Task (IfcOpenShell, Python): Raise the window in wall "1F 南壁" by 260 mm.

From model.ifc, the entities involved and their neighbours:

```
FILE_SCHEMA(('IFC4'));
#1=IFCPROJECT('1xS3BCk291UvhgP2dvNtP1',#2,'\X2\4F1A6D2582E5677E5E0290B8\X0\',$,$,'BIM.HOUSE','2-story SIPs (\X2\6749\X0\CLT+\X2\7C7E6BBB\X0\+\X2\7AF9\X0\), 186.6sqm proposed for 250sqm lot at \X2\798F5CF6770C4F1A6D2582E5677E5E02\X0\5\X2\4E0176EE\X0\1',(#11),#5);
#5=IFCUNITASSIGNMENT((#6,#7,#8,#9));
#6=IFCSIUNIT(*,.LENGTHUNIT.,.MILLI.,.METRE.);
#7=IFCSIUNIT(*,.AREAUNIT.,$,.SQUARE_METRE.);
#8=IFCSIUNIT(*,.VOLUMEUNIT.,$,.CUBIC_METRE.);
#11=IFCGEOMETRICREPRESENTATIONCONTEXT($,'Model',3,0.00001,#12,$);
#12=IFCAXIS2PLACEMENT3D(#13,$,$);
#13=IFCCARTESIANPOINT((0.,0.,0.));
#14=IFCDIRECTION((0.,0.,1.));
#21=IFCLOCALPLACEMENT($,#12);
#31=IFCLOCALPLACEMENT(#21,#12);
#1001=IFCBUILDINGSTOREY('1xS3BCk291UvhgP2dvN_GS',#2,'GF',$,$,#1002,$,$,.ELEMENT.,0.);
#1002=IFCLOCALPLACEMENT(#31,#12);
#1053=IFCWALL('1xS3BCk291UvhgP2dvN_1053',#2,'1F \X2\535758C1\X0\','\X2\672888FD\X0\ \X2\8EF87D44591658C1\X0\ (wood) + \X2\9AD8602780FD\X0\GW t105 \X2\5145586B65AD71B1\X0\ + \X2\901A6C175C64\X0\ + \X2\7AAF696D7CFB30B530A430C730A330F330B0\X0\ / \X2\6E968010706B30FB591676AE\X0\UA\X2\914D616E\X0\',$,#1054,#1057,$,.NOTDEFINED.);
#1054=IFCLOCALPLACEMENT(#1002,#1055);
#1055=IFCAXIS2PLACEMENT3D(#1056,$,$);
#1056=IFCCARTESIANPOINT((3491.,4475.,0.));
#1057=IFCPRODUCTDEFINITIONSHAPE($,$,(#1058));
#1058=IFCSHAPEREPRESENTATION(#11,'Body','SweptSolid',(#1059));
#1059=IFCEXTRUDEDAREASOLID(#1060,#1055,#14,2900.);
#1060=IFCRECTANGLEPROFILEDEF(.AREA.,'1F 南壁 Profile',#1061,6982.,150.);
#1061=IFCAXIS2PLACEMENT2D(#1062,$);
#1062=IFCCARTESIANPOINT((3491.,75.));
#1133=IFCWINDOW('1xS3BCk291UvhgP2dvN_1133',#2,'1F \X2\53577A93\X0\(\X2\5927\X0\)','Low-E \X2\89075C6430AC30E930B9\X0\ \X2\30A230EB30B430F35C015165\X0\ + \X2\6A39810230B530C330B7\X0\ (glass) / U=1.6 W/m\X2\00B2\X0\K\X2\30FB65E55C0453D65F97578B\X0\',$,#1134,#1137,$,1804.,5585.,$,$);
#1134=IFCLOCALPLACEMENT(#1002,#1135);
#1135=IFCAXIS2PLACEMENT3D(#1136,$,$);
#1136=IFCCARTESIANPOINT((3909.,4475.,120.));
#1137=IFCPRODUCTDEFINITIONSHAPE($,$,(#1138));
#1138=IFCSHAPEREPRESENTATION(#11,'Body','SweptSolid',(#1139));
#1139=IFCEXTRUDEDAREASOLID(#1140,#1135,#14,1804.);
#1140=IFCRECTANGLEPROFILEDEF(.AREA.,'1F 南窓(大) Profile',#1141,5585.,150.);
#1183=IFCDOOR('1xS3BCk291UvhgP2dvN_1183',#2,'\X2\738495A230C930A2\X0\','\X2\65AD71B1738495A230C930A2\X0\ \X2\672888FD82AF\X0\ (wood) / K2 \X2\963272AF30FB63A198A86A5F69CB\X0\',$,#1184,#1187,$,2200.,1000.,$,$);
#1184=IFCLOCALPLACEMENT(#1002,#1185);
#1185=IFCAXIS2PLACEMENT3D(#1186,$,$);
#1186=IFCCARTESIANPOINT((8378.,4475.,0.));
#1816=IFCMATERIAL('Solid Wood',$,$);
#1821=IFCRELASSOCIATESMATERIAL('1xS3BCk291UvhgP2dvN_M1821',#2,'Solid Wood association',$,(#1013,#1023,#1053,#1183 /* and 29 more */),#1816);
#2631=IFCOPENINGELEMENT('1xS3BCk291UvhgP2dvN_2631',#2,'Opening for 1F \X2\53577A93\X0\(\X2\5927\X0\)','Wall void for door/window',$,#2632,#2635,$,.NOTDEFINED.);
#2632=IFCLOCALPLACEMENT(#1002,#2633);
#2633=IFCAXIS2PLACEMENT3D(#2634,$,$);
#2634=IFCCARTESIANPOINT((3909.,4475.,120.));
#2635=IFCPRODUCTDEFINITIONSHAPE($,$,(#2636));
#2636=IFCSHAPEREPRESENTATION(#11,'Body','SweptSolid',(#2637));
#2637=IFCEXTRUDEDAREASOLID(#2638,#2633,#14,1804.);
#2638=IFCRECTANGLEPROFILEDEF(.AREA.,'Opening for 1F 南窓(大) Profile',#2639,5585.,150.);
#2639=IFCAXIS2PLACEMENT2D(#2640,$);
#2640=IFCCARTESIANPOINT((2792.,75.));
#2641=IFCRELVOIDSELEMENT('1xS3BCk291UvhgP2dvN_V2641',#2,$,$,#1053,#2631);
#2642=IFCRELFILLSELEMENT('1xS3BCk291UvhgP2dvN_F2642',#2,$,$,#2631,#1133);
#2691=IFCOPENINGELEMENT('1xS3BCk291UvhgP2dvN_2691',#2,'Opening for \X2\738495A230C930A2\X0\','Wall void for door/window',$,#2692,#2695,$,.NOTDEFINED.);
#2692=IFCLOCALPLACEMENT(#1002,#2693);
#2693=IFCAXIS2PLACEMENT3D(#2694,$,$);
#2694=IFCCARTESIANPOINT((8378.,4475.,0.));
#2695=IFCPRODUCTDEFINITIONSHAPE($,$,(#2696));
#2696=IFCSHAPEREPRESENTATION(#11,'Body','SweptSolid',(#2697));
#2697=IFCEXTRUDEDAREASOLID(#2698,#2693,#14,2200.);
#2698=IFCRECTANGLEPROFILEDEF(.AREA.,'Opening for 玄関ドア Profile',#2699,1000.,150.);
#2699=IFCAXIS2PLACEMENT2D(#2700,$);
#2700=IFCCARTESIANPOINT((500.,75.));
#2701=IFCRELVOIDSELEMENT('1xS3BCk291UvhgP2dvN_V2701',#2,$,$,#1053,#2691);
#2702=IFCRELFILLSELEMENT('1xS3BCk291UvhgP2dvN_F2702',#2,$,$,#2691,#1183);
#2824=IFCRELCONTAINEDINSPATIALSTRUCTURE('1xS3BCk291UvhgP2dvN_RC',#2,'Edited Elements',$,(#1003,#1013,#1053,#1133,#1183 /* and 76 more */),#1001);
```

```python
import numpy as np
import ifcopenshell
import ifcopenshell.api.geometry
import ifcopenshell.util.placement
import ifcopenshell.util.unit

model = ifcopenshell.open("model.ifc")
unit_scale = ifcopenshell.util.unit.calculate_unit_scale(model)

window = model.by_guid("1xS3BCk291UvhgP2dvN_1133")
opening = window.FillsVoids[0].RelatingOpeningElement
dz = 260.0

shift = np.array([0.0, 0.0, dz])
# The window is not placed relative to its opening, so move both.
for product in (opening, window):
    matrix = ifcopenshell.util.placement.get_local_placement(product.ObjectPlacement)
    matrix[:3, 3] += shift
    ifcopenshell.api.geometry.edit_object_placement(model, product=product, matrix=matrix, is_si=False)

print(f"moved by {dz * unit_scale:+.3f} m")

model.write("model_rev.ifc")
```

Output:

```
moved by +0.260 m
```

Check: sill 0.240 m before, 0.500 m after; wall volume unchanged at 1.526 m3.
